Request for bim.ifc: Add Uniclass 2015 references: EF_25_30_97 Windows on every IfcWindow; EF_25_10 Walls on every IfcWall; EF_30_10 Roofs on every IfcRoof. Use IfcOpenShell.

First a look at what the model holds.

```python
import ifcopenshell

model = ifcopenshell.open("bim.ifc")
print(model.schema)
print("classifications:", [c.Name for c in model.by_type("IfcClassification")])
for ifc_class in ("IfcDoor", "IfcRoof", "IfcStair", "IfcWall", "IfcWindow"):
    print(ifc_class, len(model.by_type(ifc_class)))
```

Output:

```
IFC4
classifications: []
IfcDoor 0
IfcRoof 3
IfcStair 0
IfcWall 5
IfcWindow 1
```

```python
import ifcopenshell
import ifcopenshell.api.classification

model = ifcopenshell.open("bim.ifc")

system = ifcopenshell.api.classification.add_classification(model, classification="Uniclass 2015")

codes = {
    "IfcWindow": ("EF_25_30_97", "Windows"),
    "IfcWall": ("EF_25_10", "Walls"),
    "IfcRoof": ("EF_30_10", "Roofs"),
}
for ifc_class, (code, name) in codes.items():
    products = model.by_type(ifc_class)
    ifcopenshell.api.classification.add_reference(
        model, products=products, classification=system, identification=code, name=name
    )
    print(code, len(products))

model.write("bim_edited.ifc")
```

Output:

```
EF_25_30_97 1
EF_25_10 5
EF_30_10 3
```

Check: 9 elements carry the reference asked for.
